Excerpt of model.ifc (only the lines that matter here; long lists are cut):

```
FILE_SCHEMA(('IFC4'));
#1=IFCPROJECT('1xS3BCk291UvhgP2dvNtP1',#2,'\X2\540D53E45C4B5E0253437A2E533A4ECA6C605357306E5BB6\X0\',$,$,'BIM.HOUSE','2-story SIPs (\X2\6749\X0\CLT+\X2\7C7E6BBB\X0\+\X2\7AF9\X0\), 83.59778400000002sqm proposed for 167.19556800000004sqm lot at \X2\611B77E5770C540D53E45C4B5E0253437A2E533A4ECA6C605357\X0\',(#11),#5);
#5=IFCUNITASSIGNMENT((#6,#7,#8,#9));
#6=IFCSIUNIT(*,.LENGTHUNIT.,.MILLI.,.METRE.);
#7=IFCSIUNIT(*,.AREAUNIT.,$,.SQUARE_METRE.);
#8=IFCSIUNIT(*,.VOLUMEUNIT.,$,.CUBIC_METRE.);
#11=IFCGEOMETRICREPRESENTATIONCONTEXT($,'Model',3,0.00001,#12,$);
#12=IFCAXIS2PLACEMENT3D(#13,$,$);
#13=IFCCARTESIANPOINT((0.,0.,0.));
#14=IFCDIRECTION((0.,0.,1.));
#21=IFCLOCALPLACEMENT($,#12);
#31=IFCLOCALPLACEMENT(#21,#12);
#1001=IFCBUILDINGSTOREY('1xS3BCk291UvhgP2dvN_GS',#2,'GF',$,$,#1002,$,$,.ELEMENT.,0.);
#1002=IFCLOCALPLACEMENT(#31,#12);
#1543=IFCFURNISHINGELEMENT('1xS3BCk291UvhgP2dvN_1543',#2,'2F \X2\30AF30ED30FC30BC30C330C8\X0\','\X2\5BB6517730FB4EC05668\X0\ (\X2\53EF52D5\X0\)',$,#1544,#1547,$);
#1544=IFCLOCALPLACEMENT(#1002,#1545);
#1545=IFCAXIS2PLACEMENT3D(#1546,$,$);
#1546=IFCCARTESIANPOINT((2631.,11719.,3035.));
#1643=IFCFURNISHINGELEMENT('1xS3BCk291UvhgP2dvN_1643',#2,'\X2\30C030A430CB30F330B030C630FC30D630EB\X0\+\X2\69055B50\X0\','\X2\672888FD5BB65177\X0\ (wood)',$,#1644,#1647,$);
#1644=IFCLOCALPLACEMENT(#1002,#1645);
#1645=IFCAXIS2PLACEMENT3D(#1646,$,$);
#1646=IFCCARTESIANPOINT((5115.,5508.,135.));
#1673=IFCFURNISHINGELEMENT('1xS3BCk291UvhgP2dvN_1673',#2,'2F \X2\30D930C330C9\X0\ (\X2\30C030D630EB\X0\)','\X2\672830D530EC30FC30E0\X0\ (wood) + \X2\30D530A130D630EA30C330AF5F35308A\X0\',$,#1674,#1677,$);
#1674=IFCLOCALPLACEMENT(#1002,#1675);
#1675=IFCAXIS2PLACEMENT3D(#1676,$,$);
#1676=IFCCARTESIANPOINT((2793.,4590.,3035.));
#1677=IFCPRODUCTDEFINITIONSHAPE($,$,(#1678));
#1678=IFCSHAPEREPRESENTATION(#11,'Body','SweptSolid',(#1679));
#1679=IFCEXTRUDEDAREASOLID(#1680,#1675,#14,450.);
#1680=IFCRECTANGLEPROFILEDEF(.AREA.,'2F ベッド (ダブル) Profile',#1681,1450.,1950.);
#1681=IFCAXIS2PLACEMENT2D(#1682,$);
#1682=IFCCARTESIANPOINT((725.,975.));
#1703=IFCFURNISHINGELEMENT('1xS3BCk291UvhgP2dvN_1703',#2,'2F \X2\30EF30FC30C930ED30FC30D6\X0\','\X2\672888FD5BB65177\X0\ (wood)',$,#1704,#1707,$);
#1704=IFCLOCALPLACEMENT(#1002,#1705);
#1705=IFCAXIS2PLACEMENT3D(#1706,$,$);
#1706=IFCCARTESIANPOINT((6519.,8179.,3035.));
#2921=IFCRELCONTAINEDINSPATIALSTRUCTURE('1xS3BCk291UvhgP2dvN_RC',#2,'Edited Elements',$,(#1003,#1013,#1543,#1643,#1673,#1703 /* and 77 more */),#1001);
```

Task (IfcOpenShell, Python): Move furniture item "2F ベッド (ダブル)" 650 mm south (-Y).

```python
import ifcopenshell
import ifcopenshell.api.geometry
import ifcopenshell.util.placement
import ifcopenshell.util.unit

model = ifcopenshell.open("model.ifc")
unit_scale = ifcopenshell.util.unit.calculate_unit_scale(model)

item = model.by_id(1673)
matrix = ifcopenshell.util.placement.get_local_placement(item.ObjectPlacement)
matrix[1, 3] -= 0.65 / unit_scale
ifcopenshell.api.geometry.edit_object_placement(model, product=item, matrix=matrix, is_si=False)

print(ifcopenshell.util.placement.get_local_placement(item.ObjectPlacement).round(3) + 0.0)

model.write("model_rev.ifc")
```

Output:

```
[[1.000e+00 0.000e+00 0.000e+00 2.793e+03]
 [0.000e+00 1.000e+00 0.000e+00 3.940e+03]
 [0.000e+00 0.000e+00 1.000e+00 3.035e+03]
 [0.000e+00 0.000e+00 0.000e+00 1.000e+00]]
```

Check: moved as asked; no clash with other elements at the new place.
